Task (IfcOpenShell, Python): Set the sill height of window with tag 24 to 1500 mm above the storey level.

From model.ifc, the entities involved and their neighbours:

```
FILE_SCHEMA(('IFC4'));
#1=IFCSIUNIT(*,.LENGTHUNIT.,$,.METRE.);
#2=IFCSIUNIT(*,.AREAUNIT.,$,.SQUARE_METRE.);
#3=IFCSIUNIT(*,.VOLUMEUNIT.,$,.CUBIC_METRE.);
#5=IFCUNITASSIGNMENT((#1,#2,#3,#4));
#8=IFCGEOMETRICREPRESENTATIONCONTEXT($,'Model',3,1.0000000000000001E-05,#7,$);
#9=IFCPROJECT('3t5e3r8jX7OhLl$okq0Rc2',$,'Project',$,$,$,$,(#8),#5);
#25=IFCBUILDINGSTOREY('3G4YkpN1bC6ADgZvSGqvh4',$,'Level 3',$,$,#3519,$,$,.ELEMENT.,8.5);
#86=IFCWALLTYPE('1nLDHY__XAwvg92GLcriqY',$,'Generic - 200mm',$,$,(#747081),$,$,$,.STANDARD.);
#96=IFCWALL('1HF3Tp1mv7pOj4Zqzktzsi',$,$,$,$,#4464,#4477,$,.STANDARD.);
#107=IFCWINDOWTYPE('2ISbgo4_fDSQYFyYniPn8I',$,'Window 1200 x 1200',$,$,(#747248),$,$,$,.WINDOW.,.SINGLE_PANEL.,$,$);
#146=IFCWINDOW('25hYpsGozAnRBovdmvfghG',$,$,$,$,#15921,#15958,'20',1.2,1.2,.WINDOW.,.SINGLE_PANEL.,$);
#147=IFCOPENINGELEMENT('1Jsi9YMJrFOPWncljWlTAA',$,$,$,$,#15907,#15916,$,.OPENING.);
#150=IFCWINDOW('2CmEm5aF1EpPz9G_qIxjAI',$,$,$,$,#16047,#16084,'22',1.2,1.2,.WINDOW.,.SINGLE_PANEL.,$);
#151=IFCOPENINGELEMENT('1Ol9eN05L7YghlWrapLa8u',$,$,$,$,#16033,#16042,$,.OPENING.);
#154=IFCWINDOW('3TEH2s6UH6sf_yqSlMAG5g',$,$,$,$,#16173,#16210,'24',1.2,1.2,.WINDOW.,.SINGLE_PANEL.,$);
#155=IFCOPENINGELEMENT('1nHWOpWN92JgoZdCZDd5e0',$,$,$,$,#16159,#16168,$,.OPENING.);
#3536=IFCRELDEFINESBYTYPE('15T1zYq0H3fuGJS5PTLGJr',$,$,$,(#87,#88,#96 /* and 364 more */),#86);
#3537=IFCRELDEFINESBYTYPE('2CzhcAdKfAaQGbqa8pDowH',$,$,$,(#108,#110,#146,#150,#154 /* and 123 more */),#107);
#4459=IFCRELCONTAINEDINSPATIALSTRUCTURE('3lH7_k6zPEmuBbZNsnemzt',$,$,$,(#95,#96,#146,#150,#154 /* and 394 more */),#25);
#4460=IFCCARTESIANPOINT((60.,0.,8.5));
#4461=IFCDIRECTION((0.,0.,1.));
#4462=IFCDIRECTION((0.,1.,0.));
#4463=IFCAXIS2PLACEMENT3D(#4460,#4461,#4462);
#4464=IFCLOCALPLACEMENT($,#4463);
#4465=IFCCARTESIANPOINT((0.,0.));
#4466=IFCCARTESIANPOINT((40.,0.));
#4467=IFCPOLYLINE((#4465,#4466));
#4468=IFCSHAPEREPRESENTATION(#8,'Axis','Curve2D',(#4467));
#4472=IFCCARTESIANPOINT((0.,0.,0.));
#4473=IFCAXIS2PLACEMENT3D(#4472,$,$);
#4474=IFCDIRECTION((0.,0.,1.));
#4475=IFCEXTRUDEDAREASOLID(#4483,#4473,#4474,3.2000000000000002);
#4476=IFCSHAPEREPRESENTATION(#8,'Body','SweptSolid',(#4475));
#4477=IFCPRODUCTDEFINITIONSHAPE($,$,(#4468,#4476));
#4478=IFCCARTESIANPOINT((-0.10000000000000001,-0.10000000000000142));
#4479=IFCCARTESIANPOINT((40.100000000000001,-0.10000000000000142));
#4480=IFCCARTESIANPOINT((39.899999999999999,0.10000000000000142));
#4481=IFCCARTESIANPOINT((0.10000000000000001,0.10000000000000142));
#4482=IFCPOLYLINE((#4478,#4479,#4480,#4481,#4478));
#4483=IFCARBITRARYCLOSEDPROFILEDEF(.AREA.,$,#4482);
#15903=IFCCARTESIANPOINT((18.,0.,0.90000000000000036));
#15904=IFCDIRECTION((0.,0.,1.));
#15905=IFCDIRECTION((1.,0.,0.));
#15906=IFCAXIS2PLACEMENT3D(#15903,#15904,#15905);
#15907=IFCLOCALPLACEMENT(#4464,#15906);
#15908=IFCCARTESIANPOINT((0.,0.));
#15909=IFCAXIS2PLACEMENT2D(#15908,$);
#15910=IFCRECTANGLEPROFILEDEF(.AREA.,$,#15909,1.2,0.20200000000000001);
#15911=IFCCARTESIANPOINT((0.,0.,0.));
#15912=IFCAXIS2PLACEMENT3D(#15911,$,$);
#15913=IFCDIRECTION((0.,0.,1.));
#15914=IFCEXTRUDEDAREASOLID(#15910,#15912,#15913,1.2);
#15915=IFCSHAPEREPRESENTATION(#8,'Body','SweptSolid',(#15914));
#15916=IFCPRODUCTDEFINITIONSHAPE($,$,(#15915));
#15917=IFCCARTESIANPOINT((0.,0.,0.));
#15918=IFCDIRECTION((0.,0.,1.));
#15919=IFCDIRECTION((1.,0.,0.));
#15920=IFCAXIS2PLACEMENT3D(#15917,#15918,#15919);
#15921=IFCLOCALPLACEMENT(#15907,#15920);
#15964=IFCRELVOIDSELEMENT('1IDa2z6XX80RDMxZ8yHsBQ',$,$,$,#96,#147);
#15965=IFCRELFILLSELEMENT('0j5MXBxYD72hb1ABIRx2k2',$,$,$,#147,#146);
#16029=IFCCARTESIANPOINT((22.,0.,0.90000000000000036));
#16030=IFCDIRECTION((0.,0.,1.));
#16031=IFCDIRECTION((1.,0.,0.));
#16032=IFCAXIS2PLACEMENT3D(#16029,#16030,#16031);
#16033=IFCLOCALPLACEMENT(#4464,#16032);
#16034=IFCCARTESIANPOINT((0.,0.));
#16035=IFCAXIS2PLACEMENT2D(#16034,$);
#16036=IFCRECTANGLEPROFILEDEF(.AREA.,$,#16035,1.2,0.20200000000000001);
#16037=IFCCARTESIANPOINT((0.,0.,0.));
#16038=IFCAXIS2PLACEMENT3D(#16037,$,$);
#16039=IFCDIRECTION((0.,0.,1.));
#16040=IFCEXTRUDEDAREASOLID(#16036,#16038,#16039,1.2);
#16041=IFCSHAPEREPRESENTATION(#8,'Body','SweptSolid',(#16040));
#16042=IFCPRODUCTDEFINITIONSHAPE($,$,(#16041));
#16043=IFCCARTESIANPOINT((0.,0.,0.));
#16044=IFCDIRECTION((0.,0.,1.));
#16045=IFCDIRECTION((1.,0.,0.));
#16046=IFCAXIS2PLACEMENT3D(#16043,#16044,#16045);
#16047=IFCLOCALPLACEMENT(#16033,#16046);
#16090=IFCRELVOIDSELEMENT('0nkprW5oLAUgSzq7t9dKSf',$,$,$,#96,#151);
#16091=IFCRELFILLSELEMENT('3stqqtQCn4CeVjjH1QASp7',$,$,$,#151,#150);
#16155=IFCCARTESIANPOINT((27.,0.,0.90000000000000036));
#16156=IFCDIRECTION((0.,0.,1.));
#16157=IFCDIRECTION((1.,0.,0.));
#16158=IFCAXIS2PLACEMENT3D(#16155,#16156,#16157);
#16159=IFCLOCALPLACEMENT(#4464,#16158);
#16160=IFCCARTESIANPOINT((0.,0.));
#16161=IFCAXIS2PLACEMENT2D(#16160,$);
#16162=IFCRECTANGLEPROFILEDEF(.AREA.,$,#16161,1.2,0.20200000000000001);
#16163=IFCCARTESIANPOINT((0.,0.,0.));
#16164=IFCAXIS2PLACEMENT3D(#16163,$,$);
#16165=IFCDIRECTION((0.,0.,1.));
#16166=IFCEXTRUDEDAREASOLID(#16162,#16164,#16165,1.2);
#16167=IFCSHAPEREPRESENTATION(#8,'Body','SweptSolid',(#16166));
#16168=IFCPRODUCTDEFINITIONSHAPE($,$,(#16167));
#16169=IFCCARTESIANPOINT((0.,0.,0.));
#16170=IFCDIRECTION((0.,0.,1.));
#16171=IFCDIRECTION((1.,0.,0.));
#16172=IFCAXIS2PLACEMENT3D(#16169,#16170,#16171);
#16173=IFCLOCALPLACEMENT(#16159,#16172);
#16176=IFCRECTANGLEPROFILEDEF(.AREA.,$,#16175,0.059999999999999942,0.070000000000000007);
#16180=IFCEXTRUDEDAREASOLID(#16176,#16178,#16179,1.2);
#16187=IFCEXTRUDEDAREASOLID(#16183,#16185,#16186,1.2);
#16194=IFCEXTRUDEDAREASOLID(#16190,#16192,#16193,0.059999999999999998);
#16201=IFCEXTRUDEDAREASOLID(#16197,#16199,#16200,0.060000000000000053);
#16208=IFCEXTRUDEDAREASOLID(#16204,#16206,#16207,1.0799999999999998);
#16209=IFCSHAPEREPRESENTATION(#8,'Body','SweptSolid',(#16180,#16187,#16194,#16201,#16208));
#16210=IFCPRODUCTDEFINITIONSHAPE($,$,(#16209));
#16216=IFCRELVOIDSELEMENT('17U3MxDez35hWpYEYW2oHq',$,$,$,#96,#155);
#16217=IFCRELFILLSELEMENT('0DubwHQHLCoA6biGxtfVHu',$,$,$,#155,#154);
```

```python
import numpy as np
import ifcopenshell
import ifcopenshell.api.geometry
import ifcopenshell.geom
import ifcopenshell.util.element
import ifcopenshell.util.placement
import ifcopenshell.util.shape
import ifcopenshell.util.unit

model = ifcopenshell.open("model.ifc")
unit_scale = ifcopenshell.util.unit.calculate_unit_scale(model)

window = model.by_guid("3TEH2s6UH6sf_yqSlMAG5g")
opening = window.FillsVoids[0].RelatingOpeningElement
storey = ifcopenshell.util.element.get_container(window, ifc_class="IfcBuildingStorey")
level = ifcopenshell.util.placement.get_local_placement(storey.ObjectPlacement)[2, 3]

# The opening's origin need not be at the sill, so measure its lowest point.
shape = ifcopenshell.geom.create_shape(ifcopenshell.geom.settings(), opening)
bottom = ifcopenshell.util.shape.get_shape_bottom_elevation(shape, shape.geometry) / unit_scale
dz = level + 1.5 - bottom

shift = np.array([0.0, 0.0, dz])
# The window is placed relative to its opening, so it follows when the opening moves.
matrix = ifcopenshell.util.placement.get_local_placement(opening.ObjectPlacement)
matrix[:3, 3] += shift
ifcopenshell.api.geometry.edit_object_placement(
    model, product=opening, matrix=matrix, is_si=False, should_transform_children=True
)

print(f"moved by {dz * unit_scale:+.3f} m")

model.write("model-out.ifc")
```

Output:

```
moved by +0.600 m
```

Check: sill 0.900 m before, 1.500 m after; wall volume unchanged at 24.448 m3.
